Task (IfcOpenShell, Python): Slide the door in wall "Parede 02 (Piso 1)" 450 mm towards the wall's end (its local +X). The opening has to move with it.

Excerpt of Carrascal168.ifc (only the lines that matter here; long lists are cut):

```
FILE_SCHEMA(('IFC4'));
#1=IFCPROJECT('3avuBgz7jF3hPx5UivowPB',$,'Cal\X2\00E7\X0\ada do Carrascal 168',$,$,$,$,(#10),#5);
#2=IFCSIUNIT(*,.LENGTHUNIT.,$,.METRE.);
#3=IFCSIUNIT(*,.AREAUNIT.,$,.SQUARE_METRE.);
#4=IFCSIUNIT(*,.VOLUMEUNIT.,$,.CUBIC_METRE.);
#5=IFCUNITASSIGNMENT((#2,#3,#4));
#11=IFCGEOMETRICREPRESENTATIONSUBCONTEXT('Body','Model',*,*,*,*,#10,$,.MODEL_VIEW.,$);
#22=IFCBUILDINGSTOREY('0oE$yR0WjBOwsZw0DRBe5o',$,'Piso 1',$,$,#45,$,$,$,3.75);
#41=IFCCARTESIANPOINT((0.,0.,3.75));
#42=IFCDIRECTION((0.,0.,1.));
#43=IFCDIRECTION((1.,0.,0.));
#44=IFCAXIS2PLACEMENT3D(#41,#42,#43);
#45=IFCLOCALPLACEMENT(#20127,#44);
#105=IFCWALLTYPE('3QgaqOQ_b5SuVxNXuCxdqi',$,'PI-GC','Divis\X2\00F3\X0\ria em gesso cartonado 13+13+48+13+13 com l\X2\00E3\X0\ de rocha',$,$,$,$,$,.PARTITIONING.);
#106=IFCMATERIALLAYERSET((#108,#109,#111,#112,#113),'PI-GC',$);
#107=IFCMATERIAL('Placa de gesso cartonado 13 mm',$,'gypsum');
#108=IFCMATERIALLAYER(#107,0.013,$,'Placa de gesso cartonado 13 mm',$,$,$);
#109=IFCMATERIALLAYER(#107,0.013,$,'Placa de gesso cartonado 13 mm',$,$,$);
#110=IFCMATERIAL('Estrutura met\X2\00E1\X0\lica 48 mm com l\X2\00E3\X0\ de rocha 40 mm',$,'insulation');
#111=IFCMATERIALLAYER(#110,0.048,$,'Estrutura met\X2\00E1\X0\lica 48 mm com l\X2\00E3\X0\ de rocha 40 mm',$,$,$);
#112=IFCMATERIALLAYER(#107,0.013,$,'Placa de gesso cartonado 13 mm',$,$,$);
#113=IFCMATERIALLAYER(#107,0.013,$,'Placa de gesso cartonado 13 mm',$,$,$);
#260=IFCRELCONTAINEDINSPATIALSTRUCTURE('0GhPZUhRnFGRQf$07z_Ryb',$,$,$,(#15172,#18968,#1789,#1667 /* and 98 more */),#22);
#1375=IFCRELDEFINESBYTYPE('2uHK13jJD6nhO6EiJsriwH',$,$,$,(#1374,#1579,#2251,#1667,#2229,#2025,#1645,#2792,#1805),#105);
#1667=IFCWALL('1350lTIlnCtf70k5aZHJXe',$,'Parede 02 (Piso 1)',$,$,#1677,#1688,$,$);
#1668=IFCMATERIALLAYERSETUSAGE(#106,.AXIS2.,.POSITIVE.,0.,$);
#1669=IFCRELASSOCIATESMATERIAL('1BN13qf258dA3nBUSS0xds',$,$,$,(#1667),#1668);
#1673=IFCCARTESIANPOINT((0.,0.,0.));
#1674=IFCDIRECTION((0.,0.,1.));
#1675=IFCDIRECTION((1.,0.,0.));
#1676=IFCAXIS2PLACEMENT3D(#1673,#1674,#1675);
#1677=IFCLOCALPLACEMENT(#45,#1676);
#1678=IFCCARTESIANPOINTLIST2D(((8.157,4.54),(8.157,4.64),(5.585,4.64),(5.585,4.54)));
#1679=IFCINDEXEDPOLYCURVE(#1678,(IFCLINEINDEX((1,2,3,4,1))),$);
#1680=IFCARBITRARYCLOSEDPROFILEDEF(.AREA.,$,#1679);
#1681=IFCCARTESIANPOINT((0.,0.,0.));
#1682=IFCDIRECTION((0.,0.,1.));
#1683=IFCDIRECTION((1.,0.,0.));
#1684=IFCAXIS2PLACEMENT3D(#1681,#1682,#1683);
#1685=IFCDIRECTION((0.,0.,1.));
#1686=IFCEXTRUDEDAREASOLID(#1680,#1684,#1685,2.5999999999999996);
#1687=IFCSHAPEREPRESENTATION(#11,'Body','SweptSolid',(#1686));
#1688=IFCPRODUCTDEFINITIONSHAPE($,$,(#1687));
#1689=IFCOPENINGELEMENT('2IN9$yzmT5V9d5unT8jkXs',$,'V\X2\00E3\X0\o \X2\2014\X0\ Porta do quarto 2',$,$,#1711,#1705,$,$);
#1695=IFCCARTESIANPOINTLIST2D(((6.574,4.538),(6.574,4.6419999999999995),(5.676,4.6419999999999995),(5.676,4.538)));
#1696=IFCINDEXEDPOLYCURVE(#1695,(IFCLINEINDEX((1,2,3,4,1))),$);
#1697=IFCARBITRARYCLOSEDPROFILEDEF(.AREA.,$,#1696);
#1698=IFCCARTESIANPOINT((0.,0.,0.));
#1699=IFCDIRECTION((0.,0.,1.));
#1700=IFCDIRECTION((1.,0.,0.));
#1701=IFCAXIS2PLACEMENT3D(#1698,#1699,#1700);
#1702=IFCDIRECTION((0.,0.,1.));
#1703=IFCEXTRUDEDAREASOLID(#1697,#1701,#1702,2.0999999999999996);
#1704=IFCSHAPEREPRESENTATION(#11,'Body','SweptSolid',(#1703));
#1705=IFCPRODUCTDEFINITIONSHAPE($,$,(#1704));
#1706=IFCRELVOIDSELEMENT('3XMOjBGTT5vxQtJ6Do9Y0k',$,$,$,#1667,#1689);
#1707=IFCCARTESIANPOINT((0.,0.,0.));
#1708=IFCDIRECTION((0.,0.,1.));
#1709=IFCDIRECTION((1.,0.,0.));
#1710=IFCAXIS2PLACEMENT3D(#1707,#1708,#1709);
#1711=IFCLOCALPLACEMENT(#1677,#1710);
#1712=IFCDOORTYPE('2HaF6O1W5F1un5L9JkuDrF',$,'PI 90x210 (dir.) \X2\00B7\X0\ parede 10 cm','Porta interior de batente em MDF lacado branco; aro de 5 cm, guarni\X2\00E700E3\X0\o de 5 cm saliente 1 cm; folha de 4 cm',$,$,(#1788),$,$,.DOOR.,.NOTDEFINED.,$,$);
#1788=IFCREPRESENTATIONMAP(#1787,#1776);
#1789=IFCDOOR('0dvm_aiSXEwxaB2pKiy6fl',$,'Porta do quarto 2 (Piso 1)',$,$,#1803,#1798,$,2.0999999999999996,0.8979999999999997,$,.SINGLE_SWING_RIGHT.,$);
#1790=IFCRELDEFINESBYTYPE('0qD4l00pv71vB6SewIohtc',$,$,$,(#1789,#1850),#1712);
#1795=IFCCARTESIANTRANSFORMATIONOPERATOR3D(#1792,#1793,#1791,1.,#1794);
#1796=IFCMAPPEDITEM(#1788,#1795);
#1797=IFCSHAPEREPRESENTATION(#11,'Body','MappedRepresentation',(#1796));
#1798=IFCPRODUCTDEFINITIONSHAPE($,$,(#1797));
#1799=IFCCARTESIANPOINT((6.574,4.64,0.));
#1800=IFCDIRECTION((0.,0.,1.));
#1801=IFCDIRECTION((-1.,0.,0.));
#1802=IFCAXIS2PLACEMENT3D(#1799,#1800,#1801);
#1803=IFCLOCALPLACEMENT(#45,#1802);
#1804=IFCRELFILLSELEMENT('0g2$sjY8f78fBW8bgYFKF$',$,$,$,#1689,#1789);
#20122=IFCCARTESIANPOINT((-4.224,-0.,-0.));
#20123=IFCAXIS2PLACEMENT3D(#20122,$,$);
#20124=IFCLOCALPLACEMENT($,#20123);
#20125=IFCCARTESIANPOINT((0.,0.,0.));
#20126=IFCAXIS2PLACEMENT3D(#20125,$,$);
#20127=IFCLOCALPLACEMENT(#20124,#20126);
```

```python
import ifcopenshell
import ifcopenshell.api.geometry
import ifcopenshell.util.placement
import ifcopenshell.util.unit

model = ifcopenshell.open("Carrascal168.ifc")
unit_scale = ifcopenshell.util.unit.calculate_unit_scale(model)

door = model.by_guid("0dvm_aiSXEwxaB2pKiy6fl")
opening = door.FillsVoids[0].RelatingOpeningElement
wall = opening.VoidsElements[0].RelatingBuildingElement

wall_matrix = ifcopenshell.util.placement.get_local_placement(wall.ObjectPlacement)
shift = wall_matrix[:3, 0] * 0.45 / unit_scale
before = ifcopenshell.util.placement.get_local_placement(door.ObjectPlacement)[:3, 3].copy()

# The door is not placed relative to its opening, so move both.
for product in (opening, door):
    matrix = ifcopenshell.util.placement.get_local_placement(product.ObjectPlacement)
    matrix[:3, 3] += shift
    ifcopenshell.api.geometry.edit_object_placement(model, product=product, matrix=matrix, is_si=False)

after = ifcopenshell.util.placement.get_local_placement(door.ObjectPlacement)[:3, 3]
print("door moved by", (after - before).round(3) + 0.0)

model.write("Carrascal168_updated.ifc")
```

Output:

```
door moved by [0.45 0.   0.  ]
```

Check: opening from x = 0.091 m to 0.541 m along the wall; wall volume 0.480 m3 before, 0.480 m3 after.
